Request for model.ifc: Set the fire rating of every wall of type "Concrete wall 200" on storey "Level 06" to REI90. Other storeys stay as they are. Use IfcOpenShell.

First a look at what the model holds.

```python
import ifcopenshell
import ifcopenshell.util.element

model = ifcopenshell.open("model.ifc")
print(model.schema)
storey = next(s for s in model.by_type("IfcBuildingStorey") if s.Name == "Level 06")
walls = [e for e in ifcopenshell.util.element.get_decomposition(storey) if e.is_a("IfcWall")]
seen = {}
for e in walls:
    element_type = ifcopenshell.util.element.get_type(e)
    key = (element_type.Name if element_type != e and element_type else None, ifcopenshell.util.element.get_pset(e, "Pset_WallCommon", "FireRating"))
    seen[key] = seen.get(key, 0) + 1
for (name, value), count in sorted(seen.items(), key=str):
    print(count, "x", name, "|", value)
```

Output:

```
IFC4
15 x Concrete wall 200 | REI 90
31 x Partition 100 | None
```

```python
import ifcopenshell
import ifcopenshell.api.pset
import ifcopenshell.util.element

model = ifcopenshell.open("model.ifc")

storey = next(s for s in model.by_type("IfcBuildingStorey") if s.Name == "Level 06")
walls = [e for e in ifcopenshell.util.element.get_decomposition(storey) if e.is_a("IfcWall")]

count = 0
for e in walls:
    element_type = ifcopenshell.util.element.get_type(e)
    if element_type in (None, e) or element_type.Name != "Concrete wall 200":
        continue
    found = ifcopenshell.util.element.get_pset(e, "Pset_WallCommon", should_inherit=False)
    if found:
        pset = model.by_id(found["id"])
        if len(ifcopenshell.util.element.get_elements_by_pset(pset)) > 1:
            pset = ifcopenshell.api.pset.unshare_pset(model, products=[e], pset=pset)[0]
    else:
        pset = ifcopenshell.api.pset.add_pset(model, product=e, name="Pset_WallCommon")
    ifcopenshell.api.pset.edit_pset(model, pset=pset, properties={"FireRating": "REI90"})
    count += 1

print(count, "walls updated")

model.write("model_v2.ifc")
```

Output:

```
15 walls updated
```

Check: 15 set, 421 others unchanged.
